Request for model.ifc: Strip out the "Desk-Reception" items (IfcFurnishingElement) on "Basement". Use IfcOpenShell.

First a look at what the model holds.

```python
import ifcopenshell
import ifcopenshell.util.element

model = ifcopenshell.open("model.ifc")
print(model.schema)
storey = next(s for s in model.by_type("IfcBuildingStorey") if s.Name == "Basement")
furniture = [e for e in ifcopenshell.util.element.get_decomposition(storey) if e.is_a("IfcFurnishingElement")]
seen = {}
for e in furniture:
    element_type = ifcopenshell.util.element.get_type(e)
    name = element_type.Name if element_type not in (None, e) else None
    seen[name] = seen.get(name, 0) + 1
for name, count in sorted(seen.items(), key=str):
    print(count, "x", name)
```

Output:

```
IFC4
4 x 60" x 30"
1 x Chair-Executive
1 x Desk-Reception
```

```python
import ifcopenshell
import ifcopenshell.api.root
import ifcopenshell.util.element

model = ifcopenshell.open("model.ifc")

storey = next(s for s in model.by_type("IfcBuildingStorey") if s.Name == "Basement")
furniture = [e for e in ifcopenshell.util.element.get_decomposition(storey) if e.is_a("IfcFurnishingElement")]
targets = [e for e in furniture if (t := ifcopenshell.util.element.get_type(e)) not in (None, e) and t.Name == "Desk-Reception"]

for e in targets:
    ifcopenshell.api.root.remove_product(model, product=e)
print(len(targets), "removed")

model.write("model-out.ifc")
```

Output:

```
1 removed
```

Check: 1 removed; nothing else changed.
